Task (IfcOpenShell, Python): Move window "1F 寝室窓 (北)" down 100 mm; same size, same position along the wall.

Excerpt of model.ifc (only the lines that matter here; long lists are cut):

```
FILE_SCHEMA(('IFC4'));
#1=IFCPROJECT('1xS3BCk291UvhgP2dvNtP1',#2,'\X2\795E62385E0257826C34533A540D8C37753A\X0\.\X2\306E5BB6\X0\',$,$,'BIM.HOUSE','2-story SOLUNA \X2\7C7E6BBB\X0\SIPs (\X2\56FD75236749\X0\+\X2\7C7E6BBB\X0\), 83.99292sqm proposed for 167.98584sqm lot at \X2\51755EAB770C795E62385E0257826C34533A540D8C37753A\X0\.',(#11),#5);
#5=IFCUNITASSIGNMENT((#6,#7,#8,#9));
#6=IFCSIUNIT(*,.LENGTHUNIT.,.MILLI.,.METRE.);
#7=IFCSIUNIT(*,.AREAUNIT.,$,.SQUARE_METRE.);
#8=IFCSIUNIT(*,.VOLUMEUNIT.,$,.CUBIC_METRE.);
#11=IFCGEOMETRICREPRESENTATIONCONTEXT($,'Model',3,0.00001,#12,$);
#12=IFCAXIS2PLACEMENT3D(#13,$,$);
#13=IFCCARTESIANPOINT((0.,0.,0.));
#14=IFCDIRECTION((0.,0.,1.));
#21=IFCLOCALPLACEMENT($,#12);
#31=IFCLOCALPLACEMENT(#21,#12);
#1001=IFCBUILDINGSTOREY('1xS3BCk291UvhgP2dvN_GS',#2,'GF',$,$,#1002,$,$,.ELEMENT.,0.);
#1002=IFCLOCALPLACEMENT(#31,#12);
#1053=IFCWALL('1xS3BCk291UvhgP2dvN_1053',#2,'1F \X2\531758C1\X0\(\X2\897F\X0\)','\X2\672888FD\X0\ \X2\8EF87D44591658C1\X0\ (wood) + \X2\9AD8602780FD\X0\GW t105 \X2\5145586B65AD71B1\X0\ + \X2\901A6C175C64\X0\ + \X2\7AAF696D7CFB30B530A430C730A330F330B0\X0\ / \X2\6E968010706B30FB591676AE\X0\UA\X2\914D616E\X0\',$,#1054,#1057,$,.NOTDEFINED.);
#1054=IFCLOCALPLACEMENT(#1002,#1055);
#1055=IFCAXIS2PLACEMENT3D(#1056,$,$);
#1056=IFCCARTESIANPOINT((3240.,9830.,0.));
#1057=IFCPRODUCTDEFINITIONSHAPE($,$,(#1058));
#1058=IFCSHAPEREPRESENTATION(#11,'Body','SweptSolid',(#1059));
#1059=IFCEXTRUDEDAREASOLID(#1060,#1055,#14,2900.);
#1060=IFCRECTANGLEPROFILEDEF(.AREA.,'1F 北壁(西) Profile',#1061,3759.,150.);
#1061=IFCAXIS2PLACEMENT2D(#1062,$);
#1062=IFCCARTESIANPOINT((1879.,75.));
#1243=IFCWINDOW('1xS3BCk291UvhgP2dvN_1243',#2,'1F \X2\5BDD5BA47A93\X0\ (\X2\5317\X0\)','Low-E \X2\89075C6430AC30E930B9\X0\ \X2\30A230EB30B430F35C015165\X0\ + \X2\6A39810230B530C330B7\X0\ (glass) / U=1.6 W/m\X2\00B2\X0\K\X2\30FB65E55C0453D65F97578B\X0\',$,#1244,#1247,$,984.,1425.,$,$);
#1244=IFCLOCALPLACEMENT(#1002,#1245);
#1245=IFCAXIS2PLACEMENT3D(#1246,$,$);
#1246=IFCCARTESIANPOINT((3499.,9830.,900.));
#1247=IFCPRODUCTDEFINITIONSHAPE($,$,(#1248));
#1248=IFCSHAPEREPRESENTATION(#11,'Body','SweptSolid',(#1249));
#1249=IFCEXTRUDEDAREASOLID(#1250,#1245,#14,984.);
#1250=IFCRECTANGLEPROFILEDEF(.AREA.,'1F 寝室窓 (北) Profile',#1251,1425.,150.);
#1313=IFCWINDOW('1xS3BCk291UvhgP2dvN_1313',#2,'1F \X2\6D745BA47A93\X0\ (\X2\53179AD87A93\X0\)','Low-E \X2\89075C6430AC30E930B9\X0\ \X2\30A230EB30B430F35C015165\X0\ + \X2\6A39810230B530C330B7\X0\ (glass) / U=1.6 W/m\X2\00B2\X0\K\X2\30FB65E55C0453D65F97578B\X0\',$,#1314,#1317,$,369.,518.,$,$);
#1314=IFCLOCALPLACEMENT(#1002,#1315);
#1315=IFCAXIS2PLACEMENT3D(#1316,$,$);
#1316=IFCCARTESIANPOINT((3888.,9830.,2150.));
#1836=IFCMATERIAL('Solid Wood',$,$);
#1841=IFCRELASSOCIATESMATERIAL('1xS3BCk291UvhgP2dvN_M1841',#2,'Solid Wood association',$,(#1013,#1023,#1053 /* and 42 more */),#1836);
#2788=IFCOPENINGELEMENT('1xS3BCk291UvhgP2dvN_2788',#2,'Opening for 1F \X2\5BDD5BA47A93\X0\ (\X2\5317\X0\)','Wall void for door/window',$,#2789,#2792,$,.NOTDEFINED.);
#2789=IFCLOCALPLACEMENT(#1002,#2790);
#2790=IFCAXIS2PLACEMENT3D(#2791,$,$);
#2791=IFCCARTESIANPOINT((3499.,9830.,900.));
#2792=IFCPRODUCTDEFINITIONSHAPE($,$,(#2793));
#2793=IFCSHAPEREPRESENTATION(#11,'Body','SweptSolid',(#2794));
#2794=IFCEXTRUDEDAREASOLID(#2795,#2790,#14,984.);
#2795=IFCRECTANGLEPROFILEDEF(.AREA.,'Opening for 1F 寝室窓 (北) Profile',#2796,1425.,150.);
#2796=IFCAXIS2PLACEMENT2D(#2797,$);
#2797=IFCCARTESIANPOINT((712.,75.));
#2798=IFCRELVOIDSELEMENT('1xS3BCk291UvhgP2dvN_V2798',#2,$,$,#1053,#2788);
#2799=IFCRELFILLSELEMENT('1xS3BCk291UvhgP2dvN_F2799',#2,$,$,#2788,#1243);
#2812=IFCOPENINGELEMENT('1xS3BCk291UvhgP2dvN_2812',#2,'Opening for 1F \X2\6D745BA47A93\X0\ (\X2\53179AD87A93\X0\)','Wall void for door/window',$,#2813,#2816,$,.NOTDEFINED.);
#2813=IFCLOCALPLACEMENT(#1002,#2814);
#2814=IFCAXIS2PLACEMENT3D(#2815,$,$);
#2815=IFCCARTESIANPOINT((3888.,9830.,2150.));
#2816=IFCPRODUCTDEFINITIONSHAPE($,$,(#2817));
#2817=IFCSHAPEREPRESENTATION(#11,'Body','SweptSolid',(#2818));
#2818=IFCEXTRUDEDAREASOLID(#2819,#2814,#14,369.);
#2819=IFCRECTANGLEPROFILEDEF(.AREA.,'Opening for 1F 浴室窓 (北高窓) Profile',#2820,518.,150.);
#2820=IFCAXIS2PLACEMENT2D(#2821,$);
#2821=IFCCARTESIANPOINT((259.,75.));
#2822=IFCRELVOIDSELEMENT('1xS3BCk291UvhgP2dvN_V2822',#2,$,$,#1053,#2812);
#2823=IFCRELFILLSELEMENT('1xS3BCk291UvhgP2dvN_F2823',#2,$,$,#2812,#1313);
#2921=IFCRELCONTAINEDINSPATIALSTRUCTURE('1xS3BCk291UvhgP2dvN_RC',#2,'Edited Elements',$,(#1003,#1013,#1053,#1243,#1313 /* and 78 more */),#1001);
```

```python
import numpy as np
import ifcopenshell
import ifcopenshell.api.geometry
import ifcopenshell.util.placement
import ifcopenshell.util.unit

model = ifcopenshell.open("model.ifc")
unit_scale = ifcopenshell.util.unit.calculate_unit_scale(model)

window = model.by_id(1243)
opening = window.FillsVoids[0].RelatingOpeningElement
dz = -0.1 / unit_scale

shift = np.array([0.0, 0.0, dz])
# The window is not placed relative to its opening, so move both.
for product in (opening, window):
    matrix = ifcopenshell.util.placement.get_local_placement(product.ObjectPlacement)
    matrix[:3, 3] += shift
    ifcopenshell.api.geometry.edit_object_placement(model, product=product, matrix=matrix, is_si=False)

print(f"moved by {dz * unit_scale:+.3f} m")

model.write("model-out.ifc")
```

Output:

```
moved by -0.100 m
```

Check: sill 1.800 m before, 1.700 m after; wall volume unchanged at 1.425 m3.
